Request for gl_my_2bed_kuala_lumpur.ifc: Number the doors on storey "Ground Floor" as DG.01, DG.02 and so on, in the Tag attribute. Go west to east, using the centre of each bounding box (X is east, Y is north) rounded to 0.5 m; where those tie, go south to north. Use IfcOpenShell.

First a look at what the model holds.

```python
import ifcopenshell
import ifcopenshell.util.element
import ifcopenshell.util.placement

model = ifcopenshell.open("gl_my_2bed_kuala_lumpur.ifc")
print(model.schema)
storey = next(s for s in model.by_type("IfcBuildingStorey") if s.Name == "Ground Floor")
doors = [e for e in ifcopenshell.util.element.get_decomposition(storey) if e.is_a("IfcDoor")]
for e in sorted(doors, key=lambda e: e.id()):
    origin = ifcopenshell.util.placement.get_local_placement(e.ObjectPlacement)[:3, 3]
    print(e.id(), e.Tag, e.Name, origin.round(2) + 0.0, sep=" | ")
```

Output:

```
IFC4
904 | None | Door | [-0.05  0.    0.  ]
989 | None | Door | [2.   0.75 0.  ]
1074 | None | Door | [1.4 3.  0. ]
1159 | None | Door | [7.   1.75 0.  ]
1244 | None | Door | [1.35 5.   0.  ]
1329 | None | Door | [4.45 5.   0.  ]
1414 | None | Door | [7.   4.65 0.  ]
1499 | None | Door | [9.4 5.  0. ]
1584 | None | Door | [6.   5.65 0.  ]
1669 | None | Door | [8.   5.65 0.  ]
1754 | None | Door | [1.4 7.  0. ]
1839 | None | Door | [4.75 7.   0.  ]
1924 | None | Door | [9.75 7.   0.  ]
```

```python
import ifcopenshell
import ifcopenshell.geom
import ifcopenshell.util.element
import ifcopenshell.util.shape

model = ifcopenshell.open("gl_my_2bed_kuala_lumpur.ifc")
settings = ifcopenshell.geom.settings()
settings.set("use-world-coords", True)


def centre(element):
    shape = ifcopenshell.geom.create_shape(settings, element)
    return ifcopenshell.util.shape.get_bbox_centroid(shape.geometry)


storey = next(s for s in model.by_type("IfcBuildingStorey") if s.Name == "Ground Floor")
doors = [e for e in ifcopenshell.util.element.get_decomposition(storey) if e.is_a("IfcDoor")]

# Insertion points can sit at a corner or the storey origin, so sort by the geometry (in metres).
centres = {e: centre(e) for e in doors}
doors.sort(key=lambda e: (round(centres[e][0] / 0.5), centres[e][1]))

for i, e in enumerate(doors, start=1):
    number = f"DG.{i:02d}"
    e.Tag = number
    print(e.id(), number)

model.write("gl_my_2bed_kuala_lumpur_v2.ifc")
```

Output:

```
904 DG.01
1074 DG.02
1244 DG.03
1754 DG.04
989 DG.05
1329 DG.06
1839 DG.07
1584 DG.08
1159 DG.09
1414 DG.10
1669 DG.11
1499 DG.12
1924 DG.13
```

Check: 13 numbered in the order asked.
